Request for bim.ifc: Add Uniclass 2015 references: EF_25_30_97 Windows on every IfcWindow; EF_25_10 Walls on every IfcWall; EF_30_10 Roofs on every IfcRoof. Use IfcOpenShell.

First a look at what the model holds.

```python
import ifcopenshell

model = ifcopenshell.open("bim.ifc")
print(model.schema)
print("classifications:", [c.Name for c in model.by_type("IfcClassification")])
for ifc_class in ("IfcDoor", "IfcRoof", "IfcStair", "IfcWall", "IfcWindow"):
    print(ifc_class, len(model.by_type(ifc_class)))
```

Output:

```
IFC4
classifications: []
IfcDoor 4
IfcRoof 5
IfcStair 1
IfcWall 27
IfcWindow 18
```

```python
import ifcopenshell
import ifcopenshell.api.classification

model = ifcopenshell.open("bim.ifc")

system = ifcopenshell.api.classification.add_classification(model, classification="Uniclass 2015")

codes = {
    "IfcWindow": ("EF_25_30_97", "Windows"),
    "IfcWall": ("EF_25_10", "Walls"),
    "IfcRoof": ("EF_30_10", "Roofs"),
}
for ifc_class, (code, name) in codes.items():
    products = model.by_type(ifc_class)
    ifcopenshell.api.classification.add_reference(
        model, products=products, classification=system, identification=code, name=name
    )
    print(code, len(products))

model.write("bim_v2.ifc")
```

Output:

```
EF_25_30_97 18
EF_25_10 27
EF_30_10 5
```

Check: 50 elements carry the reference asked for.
